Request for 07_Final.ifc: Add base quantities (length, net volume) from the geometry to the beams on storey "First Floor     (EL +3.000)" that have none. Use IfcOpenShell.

First a look at what the model holds.

```python
import ifcopenshell
import ifcopenshell.util.element
import ifcopenshell.util.unit

model = ifcopenshell.open("07_Final.ifc")
print(model.schema)
for unit_type in ("LENGTHUNIT", "AREAUNIT", "VOLUMEUNIT"):
    print(unit_type, ifcopenshell.util.unit.calculate_unit_scale(model, unit_type))
storey = next(s for s in model.by_type("IfcBuildingStorey") if s.Name == "First Floor     (EL +3.000)")
beams = [e for e in ifcopenshell.util.element.get_decomposition(storey) if e.is_a("IfcBeam")]
for e in sorted(beams, key=lambda e: e.id()):
    print(e.id(), e.is_a(), e.Name, list(ifcopenshell.util.element.get_psets(e, qtos_only=True)), sep=" | ")
```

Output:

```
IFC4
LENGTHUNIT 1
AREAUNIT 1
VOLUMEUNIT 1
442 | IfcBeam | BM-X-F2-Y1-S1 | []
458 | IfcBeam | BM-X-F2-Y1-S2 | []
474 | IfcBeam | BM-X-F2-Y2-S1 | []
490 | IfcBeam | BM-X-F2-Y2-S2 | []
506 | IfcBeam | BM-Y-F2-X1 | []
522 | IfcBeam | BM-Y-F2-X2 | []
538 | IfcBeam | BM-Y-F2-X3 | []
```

```python
import ifcopenshell
import ifcopenshell.api.pset
import ifcopenshell.geom
import ifcopenshell.util.element
import ifcopenshell.util.shape
import ifcopenshell.util.unit

model = ifcopenshell.open("07_Final.ifc")
unit_scale = ifcopenshell.util.unit.calculate_unit_scale(model)
volume_scale = ifcopenshell.util.unit.calculate_unit_scale(model, "VOLUMEUNIT")
settings = ifcopenshell.geom.settings()

storey = next(s for s in model.by_type("IfcBuildingStorey") if s.Name == "First Floor     (EL +3.000)")
beams = [e for e in ifcopenshell.util.element.get_decomposition(storey) if e.is_a("IfcBeam")]

for e in sorted(beams, key=lambda e: e.id()):
    if ifcopenshell.util.element.get_psets(e, qtos_only=True, should_inherit=False):
        continue
    # Geometry comes back in metres, in the element's own axes.
    shape = ifcopenshell.geom.create_shape(settings, e)
    values = {
        "Length": ifcopenshell.util.shape.get_max_xyz(shape.geometry) / unit_scale,
        "NetVolume": ifcopenshell.util.shape.get_volume(shape.geometry) / volume_scale,
    }
    qto = ifcopenshell.api.pset.add_qto(model, product=e, name="Qto_BeamBaseQuantities")
    ifcopenshell.api.pset.edit_qto(model, qto=qto, properties=values)
    print(e.id(), {k: round(v, 3) for k, v in values.items()})

model.write("07_Final_rev.ifc")
```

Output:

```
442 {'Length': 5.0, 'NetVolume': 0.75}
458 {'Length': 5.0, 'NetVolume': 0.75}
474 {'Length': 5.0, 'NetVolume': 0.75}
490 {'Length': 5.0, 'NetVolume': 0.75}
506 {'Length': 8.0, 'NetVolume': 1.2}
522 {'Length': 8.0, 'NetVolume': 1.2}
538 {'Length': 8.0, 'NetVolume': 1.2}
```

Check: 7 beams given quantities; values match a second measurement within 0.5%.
